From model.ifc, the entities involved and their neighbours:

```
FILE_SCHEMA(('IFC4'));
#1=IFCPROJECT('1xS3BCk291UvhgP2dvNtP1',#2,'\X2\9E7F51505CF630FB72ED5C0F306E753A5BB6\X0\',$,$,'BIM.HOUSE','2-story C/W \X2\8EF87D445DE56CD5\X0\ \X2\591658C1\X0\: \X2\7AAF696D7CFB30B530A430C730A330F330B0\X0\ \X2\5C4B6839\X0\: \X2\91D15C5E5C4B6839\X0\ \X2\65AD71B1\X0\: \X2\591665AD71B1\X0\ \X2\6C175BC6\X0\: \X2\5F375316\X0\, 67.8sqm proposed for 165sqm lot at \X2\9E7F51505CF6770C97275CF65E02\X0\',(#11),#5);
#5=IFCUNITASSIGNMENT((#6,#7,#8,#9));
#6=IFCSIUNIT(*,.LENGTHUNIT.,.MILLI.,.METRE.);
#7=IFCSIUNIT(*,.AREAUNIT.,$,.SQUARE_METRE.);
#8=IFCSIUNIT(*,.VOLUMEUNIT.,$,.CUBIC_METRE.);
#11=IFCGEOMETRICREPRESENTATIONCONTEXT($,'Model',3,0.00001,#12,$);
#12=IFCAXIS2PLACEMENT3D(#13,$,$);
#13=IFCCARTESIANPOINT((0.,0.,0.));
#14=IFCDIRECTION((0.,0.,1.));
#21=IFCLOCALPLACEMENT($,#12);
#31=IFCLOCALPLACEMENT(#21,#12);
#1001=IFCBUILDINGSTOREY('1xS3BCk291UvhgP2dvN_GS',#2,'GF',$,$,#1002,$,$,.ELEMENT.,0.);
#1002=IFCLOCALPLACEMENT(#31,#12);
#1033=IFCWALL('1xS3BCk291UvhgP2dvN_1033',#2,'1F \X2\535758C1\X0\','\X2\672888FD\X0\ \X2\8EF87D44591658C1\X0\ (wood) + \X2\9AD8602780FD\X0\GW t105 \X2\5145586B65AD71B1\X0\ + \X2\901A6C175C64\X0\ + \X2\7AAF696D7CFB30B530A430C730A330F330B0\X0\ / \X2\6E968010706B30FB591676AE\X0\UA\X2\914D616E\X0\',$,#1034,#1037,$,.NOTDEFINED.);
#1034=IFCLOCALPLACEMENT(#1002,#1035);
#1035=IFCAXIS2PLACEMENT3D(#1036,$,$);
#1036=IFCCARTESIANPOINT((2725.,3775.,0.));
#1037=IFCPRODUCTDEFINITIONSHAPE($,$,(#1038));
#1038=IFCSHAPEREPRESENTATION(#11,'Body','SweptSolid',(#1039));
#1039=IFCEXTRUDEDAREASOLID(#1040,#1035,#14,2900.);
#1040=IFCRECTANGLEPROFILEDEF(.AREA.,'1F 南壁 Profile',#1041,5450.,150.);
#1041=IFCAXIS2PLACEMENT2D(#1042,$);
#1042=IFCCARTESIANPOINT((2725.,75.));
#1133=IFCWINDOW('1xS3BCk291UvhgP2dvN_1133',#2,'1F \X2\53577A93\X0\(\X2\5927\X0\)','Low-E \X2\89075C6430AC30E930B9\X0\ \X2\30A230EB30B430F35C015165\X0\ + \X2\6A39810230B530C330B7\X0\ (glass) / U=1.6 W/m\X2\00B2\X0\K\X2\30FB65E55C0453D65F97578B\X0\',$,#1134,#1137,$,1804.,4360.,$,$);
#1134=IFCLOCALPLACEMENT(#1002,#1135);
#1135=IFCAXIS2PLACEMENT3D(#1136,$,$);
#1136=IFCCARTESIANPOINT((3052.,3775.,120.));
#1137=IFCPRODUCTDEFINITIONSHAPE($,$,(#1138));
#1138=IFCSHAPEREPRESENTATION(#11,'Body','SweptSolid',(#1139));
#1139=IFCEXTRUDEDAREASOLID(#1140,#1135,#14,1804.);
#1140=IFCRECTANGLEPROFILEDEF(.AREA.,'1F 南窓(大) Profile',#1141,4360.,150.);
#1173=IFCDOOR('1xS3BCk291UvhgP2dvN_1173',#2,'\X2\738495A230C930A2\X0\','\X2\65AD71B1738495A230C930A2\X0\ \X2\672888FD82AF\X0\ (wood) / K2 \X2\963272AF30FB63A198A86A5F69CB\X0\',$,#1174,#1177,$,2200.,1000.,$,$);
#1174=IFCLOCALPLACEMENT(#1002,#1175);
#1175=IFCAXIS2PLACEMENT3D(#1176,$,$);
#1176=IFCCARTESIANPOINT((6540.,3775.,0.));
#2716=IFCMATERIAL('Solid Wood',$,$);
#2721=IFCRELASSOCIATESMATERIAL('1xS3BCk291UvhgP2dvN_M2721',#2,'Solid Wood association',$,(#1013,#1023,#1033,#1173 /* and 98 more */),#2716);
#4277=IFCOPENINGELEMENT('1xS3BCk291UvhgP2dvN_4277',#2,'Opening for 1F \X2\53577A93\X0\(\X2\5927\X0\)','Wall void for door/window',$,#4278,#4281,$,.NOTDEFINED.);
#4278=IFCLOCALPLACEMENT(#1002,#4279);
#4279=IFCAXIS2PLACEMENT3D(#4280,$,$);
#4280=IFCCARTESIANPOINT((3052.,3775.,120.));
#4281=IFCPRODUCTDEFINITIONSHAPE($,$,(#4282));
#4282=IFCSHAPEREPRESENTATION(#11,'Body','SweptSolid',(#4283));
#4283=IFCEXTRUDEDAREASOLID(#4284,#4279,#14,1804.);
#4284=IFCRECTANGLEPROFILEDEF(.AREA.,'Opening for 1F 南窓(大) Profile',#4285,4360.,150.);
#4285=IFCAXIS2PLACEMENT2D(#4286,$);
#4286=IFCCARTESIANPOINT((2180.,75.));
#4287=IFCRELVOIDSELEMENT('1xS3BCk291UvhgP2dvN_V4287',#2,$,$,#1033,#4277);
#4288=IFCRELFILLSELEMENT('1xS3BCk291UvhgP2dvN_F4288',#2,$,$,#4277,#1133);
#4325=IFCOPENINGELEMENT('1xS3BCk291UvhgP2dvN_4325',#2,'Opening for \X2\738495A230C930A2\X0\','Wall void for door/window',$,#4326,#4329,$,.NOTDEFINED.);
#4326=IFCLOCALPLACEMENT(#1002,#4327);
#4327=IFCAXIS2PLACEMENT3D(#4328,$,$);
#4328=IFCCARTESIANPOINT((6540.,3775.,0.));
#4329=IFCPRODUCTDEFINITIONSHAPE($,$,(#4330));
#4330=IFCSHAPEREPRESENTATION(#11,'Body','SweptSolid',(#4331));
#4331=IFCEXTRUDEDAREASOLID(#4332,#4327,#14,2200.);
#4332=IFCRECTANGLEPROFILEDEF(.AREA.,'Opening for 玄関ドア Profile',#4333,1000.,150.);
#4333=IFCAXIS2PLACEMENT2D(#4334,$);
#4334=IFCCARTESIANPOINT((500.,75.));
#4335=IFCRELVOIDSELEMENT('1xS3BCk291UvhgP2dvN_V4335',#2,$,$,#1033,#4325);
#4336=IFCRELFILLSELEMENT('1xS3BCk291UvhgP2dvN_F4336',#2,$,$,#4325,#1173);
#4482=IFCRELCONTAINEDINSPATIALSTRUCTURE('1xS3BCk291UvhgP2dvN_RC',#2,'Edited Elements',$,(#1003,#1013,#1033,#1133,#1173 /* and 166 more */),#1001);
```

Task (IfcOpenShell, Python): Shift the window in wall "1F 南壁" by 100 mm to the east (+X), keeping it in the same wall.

```python
import ifcopenshell
import ifcopenshell.api.geometry
import ifcopenshell.util.placement

model = ifcopenshell.open("model.ifc")

window = model.by_guid("1xS3BCk291UvhgP2dvN_1133")
opening = window.FillsVoids[0].RelatingOpeningElement
wall = opening.VoidsElements[0].RelatingBuildingElement

wall_matrix = ifcopenshell.util.placement.get_local_placement(wall.ObjectPlacement)
shift = wall_matrix[:3, 0] * 100.0
before = ifcopenshell.util.placement.get_local_placement(window.ObjectPlacement)[:3, 3].copy()

# The window is not placed relative to its opening, so move both.
for product in (opening, window):
    matrix = ifcopenshell.util.placement.get_local_placement(product.ObjectPlacement)
    matrix[:3, 3] += shift
    ifcopenshell.api.geometry.edit_object_placement(model, product=product, matrix=matrix, is_si=False)

after = ifcopenshell.util.placement.get_local_placement(window.ObjectPlacement)[:3, 3]
print("window moved by", (after - before).round(3) + 0.0)

model.write("model-out.ifc")
```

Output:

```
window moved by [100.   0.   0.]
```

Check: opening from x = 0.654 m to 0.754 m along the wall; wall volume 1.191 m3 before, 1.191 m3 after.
